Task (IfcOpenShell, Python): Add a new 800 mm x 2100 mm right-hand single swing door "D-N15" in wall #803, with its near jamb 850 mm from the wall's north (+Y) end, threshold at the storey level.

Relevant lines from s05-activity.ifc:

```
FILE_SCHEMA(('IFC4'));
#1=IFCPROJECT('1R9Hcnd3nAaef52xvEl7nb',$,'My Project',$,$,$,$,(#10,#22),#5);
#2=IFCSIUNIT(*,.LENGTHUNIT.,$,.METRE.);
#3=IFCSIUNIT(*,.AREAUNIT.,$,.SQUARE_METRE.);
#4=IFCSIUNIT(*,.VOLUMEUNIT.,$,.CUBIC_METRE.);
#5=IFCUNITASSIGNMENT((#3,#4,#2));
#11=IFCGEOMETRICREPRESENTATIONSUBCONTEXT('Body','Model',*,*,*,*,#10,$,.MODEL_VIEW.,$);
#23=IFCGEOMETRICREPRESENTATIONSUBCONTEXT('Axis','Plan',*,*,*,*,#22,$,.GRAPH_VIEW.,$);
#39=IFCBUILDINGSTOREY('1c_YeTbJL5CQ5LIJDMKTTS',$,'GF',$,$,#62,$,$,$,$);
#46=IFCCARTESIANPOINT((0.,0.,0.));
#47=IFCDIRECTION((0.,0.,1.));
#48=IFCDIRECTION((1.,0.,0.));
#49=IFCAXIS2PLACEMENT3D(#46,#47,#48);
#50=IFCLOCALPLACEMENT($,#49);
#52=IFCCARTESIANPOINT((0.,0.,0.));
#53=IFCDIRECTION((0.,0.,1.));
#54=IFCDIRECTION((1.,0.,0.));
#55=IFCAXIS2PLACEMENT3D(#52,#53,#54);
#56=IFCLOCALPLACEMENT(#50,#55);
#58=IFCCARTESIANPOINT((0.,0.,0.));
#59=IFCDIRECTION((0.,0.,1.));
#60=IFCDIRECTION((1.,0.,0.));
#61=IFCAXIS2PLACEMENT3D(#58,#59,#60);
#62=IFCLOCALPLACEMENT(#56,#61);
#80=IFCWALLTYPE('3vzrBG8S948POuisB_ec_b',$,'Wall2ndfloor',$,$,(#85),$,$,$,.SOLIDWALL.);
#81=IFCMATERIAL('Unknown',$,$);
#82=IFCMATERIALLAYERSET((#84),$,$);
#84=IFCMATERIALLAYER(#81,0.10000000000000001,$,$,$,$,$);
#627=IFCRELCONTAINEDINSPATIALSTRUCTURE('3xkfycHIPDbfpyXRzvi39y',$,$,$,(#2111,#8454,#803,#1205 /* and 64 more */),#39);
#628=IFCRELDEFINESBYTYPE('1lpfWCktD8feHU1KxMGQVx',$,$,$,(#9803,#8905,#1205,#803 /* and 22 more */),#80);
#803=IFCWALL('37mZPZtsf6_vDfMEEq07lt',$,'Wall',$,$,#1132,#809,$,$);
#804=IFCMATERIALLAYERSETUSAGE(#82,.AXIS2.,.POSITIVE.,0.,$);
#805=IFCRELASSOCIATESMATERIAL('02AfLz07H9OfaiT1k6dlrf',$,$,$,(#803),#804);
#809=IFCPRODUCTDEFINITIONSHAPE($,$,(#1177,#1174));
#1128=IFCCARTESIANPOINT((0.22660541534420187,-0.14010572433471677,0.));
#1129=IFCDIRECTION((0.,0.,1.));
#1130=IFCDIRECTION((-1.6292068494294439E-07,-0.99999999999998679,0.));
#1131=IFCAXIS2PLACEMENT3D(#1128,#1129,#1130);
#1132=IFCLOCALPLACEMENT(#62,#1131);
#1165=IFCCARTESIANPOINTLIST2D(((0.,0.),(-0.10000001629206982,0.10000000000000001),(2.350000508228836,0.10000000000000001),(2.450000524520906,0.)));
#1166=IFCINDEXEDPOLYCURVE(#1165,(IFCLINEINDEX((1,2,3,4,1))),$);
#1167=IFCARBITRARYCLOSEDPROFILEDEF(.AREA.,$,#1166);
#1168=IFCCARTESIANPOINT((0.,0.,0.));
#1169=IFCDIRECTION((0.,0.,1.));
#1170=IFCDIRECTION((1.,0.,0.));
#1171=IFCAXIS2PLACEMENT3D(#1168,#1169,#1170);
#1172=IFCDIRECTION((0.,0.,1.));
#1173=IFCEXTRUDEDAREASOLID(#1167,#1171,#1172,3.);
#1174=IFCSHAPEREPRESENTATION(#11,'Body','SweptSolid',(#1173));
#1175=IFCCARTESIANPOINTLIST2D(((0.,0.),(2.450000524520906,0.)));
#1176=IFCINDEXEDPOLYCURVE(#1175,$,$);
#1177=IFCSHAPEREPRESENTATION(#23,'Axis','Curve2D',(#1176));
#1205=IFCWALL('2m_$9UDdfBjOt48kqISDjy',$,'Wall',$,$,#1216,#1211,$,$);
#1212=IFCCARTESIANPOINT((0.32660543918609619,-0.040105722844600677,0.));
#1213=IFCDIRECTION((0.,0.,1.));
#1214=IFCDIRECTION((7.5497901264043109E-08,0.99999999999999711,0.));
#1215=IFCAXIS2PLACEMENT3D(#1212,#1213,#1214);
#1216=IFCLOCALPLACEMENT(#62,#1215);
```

```python
import numpy as np
import ifcopenshell
import ifcopenshell.api.feature
import ifcopenshell.api.geometry
import ifcopenshell.api.root
import ifcopenshell.api.spatial
import ifcopenshell.geom
import ifcopenshell.util.element
import ifcopenshell.util.placement
import ifcopenshell.util.representation
import ifcopenshell.util.shape
import ifcopenshell.util.unit

model = ifcopenshell.open("s05-activity.ifc")
unit_scale = ifcopenshell.util.unit.calculate_unit_scale(model)
settings = ifcopenshell.geom.settings()


def volume(element):
    """Net volume in cubic metres, openings subtracted."""
    shape = ifcopenshell.geom.create_shape(settings, element)
    return ifcopenshell.util.shape.get_volume(shape.geometry)


wall = model.by_guid("37mZPZtsf6_vDfMEEq07lt")
storey = ifcopenshell.util.element.get_container(wall, ifc_class="IfcBuildingStorey")
context = ifcopenshell.util.representation.get_context(model, "Model", "Body", "MODEL_VIEW")
before = volume(wall)

width, height, from_end, sill = 0.8, 2.1, 0.85, 0.0  # metres

# The wall runs along its own X axis, and the end named is its -X end.
wall_shape = ifcopenshell.geom.create_shape(settings, wall)
x, y, z = ifcopenshell.util.shape.get_vertices(wall_shape.geometry).T
start = x.min() + from_end
face, thickness = float(y.min()), float(y.max() - y.min())
wall_matrix = ifcopenshell.util.placement.get_local_placement(wall.ObjectPlacement)
level = ifcopenshell.util.placement.get_local_placement(storey.ObjectPlacement)[2, 3]


def in_wall(x, y):
    """Placement at x, y metres in the wall's axes, at sill height."""
    matrix = wall_matrix.copy()
    matrix[:, 3] = wall_matrix @ np.array([x / unit_scale, y / unit_scale, 0.0, 1.0])
    matrix[2, 3] = level + sill / unit_scale
    return matrix


# Opening: a box that overshoots both wall faces by 50 mm.
opening = ifcopenshell.api.root.create_entity(model, ifc_class="IfcOpeningElement", predefined_type="OPENING")
box = ifcopenshell.api.geometry.add_wall_representation(
    model, context=context, length=width, height=height, thickness=thickness + 0.1
)
ifcopenshell.api.geometry.assign_representation(model, product=opening, representation=box)
ifcopenshell.api.geometry.edit_object_placement(model, product=opening, matrix=in_wall(start, face - 0.05), is_si=False)
ifcopenshell.api.feature.add_feature(model, feature=opening, element=wall)

door = ifcopenshell.api.root.create_entity(model, ifc_class="IfcDoor", name="D-N15", predefined_type="DOOR")
door.OverallWidth, door.OverallHeight = width / unit_scale, height / unit_scale
door.OperationType = "SINGLE_SWING_RIGHT"
body = ifcopenshell.api.geometry.add_door_representation(
    model,
    context=context,
    overall_width=door.OverallWidth,
    overall_height=door.OverallHeight,
    operation_type="SINGLE_SWING_RIGHT",
    lining_properties={"LiningDepth": thickness / unit_scale, "ThresholdDepth": thickness / unit_scale},
)
ifcopenshell.api.geometry.assign_representation(model, product=door, representation=body)
ifcopenshell.api.spatial.assign_container(model, products=[door], relating_structure=storey)
ifcopenshell.api.feature.add_filling(model, opening=opening, element=door)

# The lining spans the wall, so the door starts at the wall face.
ifcopenshell.api.geometry.edit_object_placement(model, product=door, matrix=in_wall(start, face), is_si=False)

after = volume(wall)

print(f"wall volume {before:.3f} -> {after:.3f} m3")

model.write("s05-activity_v2.ifc")
```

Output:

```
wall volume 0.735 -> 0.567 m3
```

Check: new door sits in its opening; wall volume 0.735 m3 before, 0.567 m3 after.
